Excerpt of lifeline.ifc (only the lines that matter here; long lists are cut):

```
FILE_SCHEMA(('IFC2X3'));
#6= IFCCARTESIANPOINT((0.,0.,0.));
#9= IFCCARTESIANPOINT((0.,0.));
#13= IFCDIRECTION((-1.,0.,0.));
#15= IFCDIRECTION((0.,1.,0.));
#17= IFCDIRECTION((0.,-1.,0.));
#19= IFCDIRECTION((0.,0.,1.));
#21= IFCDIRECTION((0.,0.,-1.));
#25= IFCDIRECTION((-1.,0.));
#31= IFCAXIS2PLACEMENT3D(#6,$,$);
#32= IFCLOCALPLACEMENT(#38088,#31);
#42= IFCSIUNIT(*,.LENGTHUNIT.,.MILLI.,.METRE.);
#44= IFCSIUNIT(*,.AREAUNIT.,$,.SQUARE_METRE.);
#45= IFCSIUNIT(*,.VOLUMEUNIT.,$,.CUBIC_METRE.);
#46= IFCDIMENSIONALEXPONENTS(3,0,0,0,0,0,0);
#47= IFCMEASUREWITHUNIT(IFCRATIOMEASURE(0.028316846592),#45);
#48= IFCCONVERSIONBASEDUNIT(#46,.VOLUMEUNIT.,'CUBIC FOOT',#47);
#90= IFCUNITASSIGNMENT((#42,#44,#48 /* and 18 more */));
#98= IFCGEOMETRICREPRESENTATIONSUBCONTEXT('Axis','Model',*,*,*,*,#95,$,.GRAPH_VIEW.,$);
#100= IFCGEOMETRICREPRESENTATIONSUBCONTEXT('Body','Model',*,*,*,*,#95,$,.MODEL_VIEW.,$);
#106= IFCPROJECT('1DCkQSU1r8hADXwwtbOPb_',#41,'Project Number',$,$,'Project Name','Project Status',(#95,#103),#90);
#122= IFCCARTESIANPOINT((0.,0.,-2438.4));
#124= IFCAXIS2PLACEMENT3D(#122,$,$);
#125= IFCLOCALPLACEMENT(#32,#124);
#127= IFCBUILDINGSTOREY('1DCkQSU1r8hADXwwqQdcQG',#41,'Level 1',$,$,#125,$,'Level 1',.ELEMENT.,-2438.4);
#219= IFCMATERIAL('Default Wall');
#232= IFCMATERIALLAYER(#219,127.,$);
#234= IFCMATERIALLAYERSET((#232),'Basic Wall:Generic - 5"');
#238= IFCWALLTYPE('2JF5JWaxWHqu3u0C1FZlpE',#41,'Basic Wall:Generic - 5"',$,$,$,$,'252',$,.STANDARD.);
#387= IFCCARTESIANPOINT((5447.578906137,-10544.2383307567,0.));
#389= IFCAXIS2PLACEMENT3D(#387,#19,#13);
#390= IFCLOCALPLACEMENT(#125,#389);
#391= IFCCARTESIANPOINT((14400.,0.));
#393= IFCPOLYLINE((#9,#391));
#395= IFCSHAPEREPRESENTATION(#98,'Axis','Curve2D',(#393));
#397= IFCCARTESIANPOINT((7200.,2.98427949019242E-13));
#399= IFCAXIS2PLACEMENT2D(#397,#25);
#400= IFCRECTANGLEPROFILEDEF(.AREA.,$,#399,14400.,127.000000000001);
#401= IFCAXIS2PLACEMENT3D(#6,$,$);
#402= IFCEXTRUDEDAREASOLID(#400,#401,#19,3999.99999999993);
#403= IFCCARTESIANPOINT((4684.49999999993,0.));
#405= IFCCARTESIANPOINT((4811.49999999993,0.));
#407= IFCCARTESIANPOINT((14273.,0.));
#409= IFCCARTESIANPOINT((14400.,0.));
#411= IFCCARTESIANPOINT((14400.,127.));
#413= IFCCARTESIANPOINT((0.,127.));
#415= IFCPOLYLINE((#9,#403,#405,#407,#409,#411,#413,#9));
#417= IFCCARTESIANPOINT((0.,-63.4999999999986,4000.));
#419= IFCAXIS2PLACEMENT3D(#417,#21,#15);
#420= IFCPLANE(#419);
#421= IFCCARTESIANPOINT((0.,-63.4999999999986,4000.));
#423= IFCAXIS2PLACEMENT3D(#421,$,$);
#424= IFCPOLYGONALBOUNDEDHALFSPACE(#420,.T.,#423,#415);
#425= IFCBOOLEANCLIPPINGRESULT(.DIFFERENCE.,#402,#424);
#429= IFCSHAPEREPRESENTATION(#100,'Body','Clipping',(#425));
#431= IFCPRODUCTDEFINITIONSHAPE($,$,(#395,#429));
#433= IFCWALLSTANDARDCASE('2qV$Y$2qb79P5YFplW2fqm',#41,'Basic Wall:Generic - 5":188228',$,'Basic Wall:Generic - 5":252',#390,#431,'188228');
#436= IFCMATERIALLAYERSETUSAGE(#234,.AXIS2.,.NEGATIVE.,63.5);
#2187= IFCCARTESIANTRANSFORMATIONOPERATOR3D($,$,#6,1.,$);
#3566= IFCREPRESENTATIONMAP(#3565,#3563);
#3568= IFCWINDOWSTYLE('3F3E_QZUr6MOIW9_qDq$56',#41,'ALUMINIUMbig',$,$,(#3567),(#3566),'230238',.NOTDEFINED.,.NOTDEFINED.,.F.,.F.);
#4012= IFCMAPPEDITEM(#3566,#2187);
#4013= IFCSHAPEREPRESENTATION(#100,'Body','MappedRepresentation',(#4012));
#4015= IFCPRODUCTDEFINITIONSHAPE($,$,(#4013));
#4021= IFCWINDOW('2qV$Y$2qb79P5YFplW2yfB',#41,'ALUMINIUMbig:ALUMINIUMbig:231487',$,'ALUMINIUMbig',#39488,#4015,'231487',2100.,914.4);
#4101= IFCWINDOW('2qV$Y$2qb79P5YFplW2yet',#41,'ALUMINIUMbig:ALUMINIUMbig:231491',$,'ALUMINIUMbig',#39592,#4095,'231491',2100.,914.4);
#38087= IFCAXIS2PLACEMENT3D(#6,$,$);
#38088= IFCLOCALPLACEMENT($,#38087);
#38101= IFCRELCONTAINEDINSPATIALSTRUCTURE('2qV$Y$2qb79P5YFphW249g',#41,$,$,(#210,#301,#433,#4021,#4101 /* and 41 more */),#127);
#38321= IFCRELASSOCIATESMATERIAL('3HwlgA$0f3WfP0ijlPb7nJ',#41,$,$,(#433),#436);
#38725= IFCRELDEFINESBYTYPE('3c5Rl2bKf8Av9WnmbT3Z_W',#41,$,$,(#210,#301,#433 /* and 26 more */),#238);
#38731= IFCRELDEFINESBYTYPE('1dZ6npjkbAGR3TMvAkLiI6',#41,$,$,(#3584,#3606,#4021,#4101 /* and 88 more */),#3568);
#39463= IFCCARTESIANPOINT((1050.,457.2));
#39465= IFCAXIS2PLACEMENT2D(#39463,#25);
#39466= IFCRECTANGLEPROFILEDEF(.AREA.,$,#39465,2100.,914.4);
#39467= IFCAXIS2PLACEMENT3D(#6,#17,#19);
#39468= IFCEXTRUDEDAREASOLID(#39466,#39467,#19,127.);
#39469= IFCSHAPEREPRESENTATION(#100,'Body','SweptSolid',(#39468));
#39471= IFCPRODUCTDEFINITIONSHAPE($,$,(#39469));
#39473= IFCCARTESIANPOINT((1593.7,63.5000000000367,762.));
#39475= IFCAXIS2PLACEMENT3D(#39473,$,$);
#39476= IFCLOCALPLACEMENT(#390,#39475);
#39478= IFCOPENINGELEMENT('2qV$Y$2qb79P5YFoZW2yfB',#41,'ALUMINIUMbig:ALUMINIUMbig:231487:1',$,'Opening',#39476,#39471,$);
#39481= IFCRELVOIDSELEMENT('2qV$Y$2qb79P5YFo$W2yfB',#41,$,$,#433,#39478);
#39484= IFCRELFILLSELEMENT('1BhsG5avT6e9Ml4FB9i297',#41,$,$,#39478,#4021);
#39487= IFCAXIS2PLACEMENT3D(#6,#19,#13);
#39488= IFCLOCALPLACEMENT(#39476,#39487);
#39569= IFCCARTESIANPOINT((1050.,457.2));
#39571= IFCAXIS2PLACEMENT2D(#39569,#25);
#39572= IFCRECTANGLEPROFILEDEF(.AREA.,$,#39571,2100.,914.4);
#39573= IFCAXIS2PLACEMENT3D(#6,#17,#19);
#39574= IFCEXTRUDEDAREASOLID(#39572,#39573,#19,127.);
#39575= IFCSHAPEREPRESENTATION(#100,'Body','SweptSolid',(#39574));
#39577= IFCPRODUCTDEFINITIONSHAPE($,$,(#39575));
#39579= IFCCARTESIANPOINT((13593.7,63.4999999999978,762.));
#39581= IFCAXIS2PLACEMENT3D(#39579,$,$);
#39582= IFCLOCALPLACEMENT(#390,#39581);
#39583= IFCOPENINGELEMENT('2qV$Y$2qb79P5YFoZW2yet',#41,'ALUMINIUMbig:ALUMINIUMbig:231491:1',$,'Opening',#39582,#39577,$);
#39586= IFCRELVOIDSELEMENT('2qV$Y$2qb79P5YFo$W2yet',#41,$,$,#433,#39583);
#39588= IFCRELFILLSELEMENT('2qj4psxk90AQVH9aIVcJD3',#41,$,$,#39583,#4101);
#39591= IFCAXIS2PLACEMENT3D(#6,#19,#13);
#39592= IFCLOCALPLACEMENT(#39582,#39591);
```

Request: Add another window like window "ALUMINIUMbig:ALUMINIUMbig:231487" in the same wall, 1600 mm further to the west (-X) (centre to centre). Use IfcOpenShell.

```python
import ifcopenshell
import ifcopenshell.api.feature
import ifcopenshell.api.geometry
import ifcopenshell.api.root
import ifcopenshell.geom
import ifcopenshell.util.element
import ifcopenshell.util.placement
import ifcopenshell.util.shape

model = ifcopenshell.open("lifeline.ifc")
settings = ifcopenshell.geom.settings()


def volume(element):
    """Net volume in cubic metres, openings subtracted."""
    shape = ifcopenshell.geom.create_shape(settings, element)
    return ifcopenshell.util.shape.get_volume(shape.geometry)


def reuse_history(source, copy):
    """copy_class also copies each property set's owner history, people and application; keep the originals."""
    for rel in copy.IsDefinedBy:
        if rel.is_a("IfcRelDefinesByProperties") and (history := rel.RelatingPropertyDefinition.OwnerHistory):
            rel.RelatingPropertyDefinition.OwnerHistory = source.OwnerHistory
            ifcopenshell.util.element.remove_deep2(model, history)


window = model.by_guid("2qV$Y$2qb79P5YFplW2yfB")
opening = window.FillsVoids[0].RelatingOpeningElement
wall = opening.VoidsElements[0].RelatingBuildingElement
before = volume(wall)
shift = ifcopenshell.util.placement.get_local_placement(wall.ObjectPlacement)[:3, 0] * 1600.0

# copy_class copies the void relationship, type, container and properties, but no geometry.
new_opening = ifcopenshell.api.root.copy_class(model, product=opening)
new_opening.Representation = ifcopenshell.util.element.copy_deep(
    model, opening.Representation, exclude=["IfcGeometricRepresentationContext", "IfcRepresentationMap"]
)
new_opening.Name = "ALUMINIUMbig:ALUMINIUMbig"
new_window = ifcopenshell.api.root.copy_class(model, product=window)
new_window.Representation = ifcopenshell.util.element.copy_deep(
    model, window.Representation, exclude=["IfcGeometricRepresentationContext", "IfcRepresentationMap"]
)
new_window.Name = "ALUMINIUMbig:ALUMINIUMbig"
new_window.Tag = None
reuse_history(window, new_window)
fills = ifcopenshell.api.feature.add_filling(model, opening=new_opening, element=new_window)
fills.OwnerHistory = new_window.OwnerHistory  # required in IFC2X3

for old, new in ((opening, new_opening), (window, new_window)):
    matrix = ifcopenshell.util.placement.get_local_placement(old.ObjectPlacement)
    matrix[:3, 3] += shift
    ifcopenshell.api.geometry.edit_object_placement(model, product=new, matrix=matrix, is_si=False)

after = volume(wall)

print(f"wall volume {before:.3f} -> {after:.3f} m3")

model.write("lifeline_rev.ifc")
```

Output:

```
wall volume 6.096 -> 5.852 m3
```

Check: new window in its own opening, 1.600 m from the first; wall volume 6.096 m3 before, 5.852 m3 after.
